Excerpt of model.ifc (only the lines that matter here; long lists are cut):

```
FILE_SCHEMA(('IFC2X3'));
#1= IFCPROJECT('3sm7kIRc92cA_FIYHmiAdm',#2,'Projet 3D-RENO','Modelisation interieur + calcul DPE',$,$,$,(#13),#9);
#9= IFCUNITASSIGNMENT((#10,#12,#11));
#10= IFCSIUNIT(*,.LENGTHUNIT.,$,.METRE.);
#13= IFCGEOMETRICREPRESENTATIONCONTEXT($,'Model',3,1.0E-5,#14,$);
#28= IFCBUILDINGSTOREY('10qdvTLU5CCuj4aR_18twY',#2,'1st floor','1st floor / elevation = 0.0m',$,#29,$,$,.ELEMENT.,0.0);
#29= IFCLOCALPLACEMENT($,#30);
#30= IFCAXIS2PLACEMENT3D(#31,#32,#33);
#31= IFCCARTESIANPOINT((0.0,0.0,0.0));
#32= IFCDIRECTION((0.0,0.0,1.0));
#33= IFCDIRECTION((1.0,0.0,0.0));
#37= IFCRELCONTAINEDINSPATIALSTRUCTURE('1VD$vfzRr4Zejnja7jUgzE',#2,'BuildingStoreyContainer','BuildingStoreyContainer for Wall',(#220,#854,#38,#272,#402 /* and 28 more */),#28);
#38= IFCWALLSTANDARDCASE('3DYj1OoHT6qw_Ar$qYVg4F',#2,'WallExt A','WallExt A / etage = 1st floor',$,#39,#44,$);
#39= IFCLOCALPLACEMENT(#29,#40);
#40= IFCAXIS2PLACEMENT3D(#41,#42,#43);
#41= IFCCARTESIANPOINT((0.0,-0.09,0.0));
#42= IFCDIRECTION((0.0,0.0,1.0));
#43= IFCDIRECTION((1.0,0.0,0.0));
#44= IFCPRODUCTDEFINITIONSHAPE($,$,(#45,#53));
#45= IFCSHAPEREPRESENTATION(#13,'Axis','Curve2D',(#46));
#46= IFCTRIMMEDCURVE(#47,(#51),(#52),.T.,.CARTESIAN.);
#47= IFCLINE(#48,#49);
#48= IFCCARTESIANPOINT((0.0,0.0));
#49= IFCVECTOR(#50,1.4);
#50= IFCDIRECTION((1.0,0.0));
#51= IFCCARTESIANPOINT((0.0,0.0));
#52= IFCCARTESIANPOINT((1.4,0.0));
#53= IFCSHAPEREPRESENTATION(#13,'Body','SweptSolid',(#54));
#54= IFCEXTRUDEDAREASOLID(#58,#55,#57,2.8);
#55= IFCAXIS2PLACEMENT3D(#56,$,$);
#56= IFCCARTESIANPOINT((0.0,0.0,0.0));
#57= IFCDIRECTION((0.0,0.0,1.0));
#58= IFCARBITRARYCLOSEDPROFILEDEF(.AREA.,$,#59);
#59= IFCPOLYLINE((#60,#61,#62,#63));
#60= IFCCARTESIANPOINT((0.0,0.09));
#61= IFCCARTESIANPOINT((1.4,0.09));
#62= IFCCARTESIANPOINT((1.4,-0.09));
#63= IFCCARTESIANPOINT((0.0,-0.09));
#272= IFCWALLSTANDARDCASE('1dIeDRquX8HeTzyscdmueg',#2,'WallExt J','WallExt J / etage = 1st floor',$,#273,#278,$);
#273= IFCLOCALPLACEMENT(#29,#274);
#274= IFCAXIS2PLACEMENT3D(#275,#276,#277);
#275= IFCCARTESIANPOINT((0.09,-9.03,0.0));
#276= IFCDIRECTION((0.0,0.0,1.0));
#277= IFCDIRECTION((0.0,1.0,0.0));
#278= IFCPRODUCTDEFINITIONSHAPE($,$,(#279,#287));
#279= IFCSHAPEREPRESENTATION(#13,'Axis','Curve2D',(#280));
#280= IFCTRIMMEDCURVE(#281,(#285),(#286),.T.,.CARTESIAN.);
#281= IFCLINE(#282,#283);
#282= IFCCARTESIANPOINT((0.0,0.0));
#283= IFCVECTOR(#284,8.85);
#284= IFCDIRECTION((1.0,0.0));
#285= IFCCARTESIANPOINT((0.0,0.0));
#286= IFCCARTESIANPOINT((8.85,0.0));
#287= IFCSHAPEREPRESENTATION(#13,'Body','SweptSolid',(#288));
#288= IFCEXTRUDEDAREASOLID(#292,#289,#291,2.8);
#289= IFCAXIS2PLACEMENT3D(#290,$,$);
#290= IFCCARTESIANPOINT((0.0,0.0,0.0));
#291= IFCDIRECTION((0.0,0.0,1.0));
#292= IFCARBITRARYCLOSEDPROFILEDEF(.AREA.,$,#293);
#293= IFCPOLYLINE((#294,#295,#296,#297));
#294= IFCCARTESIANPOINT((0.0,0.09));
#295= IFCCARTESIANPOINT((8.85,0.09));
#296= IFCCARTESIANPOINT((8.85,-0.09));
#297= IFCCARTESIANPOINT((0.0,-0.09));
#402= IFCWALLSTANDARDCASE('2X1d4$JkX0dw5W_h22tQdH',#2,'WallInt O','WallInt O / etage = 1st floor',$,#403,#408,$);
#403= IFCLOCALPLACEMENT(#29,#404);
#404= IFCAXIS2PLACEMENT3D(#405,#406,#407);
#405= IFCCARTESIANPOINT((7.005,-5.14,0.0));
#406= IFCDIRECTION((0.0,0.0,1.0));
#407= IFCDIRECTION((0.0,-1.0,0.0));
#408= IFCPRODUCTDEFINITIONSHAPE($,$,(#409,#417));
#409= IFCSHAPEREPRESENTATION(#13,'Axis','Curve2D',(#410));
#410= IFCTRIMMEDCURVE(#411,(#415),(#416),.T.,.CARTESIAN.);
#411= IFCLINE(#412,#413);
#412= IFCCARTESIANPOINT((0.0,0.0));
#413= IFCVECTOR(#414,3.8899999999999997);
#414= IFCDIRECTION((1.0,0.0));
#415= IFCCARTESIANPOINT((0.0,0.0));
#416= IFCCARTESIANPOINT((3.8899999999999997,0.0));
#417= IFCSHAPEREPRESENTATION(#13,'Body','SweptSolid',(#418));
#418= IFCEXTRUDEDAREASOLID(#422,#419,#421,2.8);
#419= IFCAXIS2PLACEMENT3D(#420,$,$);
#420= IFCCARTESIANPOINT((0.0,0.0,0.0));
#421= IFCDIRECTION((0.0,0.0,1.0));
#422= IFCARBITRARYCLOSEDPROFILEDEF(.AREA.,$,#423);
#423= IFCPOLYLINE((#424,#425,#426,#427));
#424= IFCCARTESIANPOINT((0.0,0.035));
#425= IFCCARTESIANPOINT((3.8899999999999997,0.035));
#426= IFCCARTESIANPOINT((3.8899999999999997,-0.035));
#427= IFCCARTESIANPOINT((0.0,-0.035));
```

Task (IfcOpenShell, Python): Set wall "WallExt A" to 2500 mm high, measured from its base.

```python
import ifcopenshell
import ifcopenshell.geom
import ifcopenshell.util.shape
import ifcopenshell.util.unit

model = ifcopenshell.open("model.ifc")
unit_scale = ifcopenshell.util.unit.calculate_unit_scale(model)
settings = ifcopenshell.geom.settings()


def volume(element):
    """Net volume in cubic metres, openings subtracted."""
    shape = ifcopenshell.geom.create_shape(settings, element)
    return ifcopenshell.util.shape.get_volume(shape.geometry)


wall = model.by_guid("3DYj1OoHT6qw_Ar$qYVg4F")
before = volume(wall)

body = next(r for r in wall.Representation.Representations if r.RepresentationIdentifier == "Body")
solid = body.Items[0]
old_height = solid.Depth
solid.Depth = 2.5 / unit_scale
after = volume(wall)

print(f"height {old_height:g} -> {solid.Depth:g}, volume {before:.3f} -> {after:.3f} m3")

model.write("model_rev.ifc")
```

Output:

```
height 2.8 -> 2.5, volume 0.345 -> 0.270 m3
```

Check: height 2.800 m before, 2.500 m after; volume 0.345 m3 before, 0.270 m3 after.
